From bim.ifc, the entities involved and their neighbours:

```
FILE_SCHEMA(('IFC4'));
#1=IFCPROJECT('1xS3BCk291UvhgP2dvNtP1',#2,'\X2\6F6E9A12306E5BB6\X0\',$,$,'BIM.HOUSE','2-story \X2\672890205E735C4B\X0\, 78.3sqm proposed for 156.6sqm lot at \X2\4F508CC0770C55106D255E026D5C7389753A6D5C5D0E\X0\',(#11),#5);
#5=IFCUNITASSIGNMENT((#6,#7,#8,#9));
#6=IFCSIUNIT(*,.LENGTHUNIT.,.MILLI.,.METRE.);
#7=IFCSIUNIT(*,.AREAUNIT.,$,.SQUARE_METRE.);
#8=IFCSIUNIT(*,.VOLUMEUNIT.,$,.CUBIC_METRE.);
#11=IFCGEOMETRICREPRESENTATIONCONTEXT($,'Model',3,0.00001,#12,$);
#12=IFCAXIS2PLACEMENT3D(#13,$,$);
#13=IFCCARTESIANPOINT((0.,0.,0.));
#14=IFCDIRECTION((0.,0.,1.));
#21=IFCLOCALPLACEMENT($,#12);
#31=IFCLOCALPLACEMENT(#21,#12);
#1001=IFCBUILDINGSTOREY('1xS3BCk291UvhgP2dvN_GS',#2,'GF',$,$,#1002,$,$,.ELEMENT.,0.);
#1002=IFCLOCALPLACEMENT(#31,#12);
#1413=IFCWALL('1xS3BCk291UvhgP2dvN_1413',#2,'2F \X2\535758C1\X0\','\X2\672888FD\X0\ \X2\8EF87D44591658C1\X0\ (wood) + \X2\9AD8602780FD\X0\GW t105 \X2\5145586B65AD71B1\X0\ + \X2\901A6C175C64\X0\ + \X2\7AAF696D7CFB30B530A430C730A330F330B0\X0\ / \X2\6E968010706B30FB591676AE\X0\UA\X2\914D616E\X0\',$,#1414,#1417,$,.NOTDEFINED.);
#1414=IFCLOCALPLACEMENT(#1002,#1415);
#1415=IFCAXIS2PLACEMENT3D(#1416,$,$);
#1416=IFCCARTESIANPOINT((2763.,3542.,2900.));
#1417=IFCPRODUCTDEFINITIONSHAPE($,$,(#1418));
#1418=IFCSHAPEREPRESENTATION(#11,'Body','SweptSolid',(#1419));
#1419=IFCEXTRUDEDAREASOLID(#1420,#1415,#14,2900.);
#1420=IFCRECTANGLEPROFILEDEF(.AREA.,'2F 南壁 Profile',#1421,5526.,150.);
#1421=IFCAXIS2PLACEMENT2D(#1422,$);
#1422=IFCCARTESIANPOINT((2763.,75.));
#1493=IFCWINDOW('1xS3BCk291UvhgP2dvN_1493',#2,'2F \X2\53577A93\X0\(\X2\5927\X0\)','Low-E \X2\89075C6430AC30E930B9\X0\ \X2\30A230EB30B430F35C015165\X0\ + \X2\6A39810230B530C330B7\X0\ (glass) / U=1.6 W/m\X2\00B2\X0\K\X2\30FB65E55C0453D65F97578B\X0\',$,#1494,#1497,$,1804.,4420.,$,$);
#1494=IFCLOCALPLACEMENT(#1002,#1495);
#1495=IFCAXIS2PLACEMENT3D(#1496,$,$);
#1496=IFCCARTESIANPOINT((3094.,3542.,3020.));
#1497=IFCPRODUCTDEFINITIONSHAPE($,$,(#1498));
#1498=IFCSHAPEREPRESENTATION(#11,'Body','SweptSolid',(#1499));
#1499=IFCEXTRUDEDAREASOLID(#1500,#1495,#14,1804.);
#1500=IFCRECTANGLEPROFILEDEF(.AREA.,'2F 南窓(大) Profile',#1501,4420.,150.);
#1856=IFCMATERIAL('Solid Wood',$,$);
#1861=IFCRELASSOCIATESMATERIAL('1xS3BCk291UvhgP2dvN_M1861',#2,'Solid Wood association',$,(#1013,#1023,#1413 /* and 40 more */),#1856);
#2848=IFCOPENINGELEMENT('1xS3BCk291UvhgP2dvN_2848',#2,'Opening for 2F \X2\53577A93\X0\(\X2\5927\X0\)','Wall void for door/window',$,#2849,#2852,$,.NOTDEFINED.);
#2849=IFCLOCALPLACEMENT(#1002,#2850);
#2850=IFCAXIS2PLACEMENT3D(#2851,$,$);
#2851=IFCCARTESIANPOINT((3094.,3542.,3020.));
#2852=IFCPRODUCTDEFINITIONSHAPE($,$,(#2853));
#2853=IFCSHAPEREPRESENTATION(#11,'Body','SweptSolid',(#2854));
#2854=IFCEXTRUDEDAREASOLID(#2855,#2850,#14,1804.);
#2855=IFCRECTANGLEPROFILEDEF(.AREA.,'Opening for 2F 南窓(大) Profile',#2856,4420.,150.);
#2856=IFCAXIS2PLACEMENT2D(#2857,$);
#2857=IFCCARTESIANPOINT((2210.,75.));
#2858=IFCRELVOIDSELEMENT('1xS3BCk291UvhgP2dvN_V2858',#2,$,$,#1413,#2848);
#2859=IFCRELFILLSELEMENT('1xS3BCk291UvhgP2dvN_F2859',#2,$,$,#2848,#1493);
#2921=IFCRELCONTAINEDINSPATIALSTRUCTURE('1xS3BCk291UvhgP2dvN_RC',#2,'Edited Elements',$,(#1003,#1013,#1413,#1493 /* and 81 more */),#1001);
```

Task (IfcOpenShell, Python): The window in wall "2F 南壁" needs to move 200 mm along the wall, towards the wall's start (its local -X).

```python
import ifcopenshell
import ifcopenshell.api.geometry
import ifcopenshell.util.placement
import ifcopenshell.util.unit

model = ifcopenshell.open("bim.ifc")
unit_scale = ifcopenshell.util.unit.calculate_unit_scale(model)

window = model.by_id(1493)
opening = window.FillsVoids[0].RelatingOpeningElement
wall = opening.VoidsElements[0].RelatingBuildingElement

wall_matrix = ifcopenshell.util.placement.get_local_placement(wall.ObjectPlacement)
shift = wall_matrix[:3, 0] * -0.2 / unit_scale
before = ifcopenshell.util.placement.get_local_placement(window.ObjectPlacement)[:3, 3].copy()

# The window is not placed relative to its opening, so move both.
for product in (opening, window):
    matrix = ifcopenshell.util.placement.get_local_placement(product.ObjectPlacement)
    matrix[:3, 3] += shift
    ifcopenshell.api.geometry.edit_object_placement(model, product=product, matrix=matrix, is_si=False)

after = ifcopenshell.util.placement.get_local_placement(window.ObjectPlacement)[:3, 3]
print("window moved by", (after - before).round(3) + 0.0)

model.write("bim-out.ifc")
```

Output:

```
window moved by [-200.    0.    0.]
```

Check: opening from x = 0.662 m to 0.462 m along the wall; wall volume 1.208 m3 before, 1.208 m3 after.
